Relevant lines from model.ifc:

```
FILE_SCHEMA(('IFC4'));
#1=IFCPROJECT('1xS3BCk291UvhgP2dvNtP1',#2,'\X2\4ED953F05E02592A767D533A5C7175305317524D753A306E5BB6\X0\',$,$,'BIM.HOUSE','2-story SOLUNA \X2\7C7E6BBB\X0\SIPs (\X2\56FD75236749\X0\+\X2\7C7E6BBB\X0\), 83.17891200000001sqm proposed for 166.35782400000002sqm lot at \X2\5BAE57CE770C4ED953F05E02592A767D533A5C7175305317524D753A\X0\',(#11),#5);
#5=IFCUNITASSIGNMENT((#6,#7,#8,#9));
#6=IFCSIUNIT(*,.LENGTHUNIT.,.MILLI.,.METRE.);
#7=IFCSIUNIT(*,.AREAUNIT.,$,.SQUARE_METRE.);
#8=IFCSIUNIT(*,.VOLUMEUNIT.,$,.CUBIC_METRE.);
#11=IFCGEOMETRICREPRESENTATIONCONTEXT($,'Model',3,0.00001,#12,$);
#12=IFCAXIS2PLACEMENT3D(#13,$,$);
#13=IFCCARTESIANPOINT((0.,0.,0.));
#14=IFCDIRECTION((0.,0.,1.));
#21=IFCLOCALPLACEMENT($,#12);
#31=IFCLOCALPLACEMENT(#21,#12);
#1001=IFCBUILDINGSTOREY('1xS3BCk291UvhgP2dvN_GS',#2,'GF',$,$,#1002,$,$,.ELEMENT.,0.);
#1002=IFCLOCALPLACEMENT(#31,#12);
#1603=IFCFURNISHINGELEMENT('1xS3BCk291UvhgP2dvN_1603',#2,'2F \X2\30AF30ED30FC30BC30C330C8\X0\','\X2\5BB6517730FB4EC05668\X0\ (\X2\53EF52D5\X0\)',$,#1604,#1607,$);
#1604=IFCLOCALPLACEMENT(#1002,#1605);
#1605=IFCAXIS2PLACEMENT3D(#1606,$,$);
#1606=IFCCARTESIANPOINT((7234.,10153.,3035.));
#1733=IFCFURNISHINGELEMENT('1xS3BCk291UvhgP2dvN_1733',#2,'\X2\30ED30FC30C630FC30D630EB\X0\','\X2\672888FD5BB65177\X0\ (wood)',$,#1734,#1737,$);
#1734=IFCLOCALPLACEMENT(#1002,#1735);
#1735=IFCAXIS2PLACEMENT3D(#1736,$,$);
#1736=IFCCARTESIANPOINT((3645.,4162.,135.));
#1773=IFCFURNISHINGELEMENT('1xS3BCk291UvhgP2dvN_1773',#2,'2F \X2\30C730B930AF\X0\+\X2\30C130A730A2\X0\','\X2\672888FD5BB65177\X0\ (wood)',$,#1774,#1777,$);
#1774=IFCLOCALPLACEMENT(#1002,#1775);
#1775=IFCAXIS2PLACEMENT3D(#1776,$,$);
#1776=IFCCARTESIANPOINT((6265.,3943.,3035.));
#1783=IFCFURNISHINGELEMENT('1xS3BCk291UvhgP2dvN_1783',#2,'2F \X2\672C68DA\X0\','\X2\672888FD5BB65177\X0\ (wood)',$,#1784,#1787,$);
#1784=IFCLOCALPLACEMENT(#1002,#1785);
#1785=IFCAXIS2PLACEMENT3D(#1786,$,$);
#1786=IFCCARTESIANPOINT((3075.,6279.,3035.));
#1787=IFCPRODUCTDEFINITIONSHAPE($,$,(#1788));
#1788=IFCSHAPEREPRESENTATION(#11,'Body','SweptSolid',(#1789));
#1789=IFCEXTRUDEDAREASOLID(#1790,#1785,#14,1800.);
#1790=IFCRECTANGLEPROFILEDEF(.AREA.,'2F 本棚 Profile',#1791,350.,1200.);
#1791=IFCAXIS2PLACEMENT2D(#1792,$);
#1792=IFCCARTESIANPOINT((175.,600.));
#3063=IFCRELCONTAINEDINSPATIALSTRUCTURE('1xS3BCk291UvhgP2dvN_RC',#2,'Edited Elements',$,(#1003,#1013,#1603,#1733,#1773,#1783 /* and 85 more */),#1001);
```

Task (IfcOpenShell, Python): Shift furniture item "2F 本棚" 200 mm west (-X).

```python
import ifcopenshell
import ifcopenshell.api.geometry
import ifcopenshell.util.placement
import ifcopenshell.util.unit

model = ifcopenshell.open("model.ifc")
unit_scale = ifcopenshell.util.unit.calculate_unit_scale(model)

item = model.by_guid("1xS3BCk291UvhgP2dvN_1783")
matrix = ifcopenshell.util.placement.get_local_placement(item.ObjectPlacement)
matrix[0, 3] -= 0.2 / unit_scale
ifcopenshell.api.geometry.edit_object_placement(model, product=item, matrix=matrix, is_si=False)

print(ifcopenshell.util.placement.get_local_placement(item.ObjectPlacement).round(3) + 0.0)

model.write("model-out.ifc")
```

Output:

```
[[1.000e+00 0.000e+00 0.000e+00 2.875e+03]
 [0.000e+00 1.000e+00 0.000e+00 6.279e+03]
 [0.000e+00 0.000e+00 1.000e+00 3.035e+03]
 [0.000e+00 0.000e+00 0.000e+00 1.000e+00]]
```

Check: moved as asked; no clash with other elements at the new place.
